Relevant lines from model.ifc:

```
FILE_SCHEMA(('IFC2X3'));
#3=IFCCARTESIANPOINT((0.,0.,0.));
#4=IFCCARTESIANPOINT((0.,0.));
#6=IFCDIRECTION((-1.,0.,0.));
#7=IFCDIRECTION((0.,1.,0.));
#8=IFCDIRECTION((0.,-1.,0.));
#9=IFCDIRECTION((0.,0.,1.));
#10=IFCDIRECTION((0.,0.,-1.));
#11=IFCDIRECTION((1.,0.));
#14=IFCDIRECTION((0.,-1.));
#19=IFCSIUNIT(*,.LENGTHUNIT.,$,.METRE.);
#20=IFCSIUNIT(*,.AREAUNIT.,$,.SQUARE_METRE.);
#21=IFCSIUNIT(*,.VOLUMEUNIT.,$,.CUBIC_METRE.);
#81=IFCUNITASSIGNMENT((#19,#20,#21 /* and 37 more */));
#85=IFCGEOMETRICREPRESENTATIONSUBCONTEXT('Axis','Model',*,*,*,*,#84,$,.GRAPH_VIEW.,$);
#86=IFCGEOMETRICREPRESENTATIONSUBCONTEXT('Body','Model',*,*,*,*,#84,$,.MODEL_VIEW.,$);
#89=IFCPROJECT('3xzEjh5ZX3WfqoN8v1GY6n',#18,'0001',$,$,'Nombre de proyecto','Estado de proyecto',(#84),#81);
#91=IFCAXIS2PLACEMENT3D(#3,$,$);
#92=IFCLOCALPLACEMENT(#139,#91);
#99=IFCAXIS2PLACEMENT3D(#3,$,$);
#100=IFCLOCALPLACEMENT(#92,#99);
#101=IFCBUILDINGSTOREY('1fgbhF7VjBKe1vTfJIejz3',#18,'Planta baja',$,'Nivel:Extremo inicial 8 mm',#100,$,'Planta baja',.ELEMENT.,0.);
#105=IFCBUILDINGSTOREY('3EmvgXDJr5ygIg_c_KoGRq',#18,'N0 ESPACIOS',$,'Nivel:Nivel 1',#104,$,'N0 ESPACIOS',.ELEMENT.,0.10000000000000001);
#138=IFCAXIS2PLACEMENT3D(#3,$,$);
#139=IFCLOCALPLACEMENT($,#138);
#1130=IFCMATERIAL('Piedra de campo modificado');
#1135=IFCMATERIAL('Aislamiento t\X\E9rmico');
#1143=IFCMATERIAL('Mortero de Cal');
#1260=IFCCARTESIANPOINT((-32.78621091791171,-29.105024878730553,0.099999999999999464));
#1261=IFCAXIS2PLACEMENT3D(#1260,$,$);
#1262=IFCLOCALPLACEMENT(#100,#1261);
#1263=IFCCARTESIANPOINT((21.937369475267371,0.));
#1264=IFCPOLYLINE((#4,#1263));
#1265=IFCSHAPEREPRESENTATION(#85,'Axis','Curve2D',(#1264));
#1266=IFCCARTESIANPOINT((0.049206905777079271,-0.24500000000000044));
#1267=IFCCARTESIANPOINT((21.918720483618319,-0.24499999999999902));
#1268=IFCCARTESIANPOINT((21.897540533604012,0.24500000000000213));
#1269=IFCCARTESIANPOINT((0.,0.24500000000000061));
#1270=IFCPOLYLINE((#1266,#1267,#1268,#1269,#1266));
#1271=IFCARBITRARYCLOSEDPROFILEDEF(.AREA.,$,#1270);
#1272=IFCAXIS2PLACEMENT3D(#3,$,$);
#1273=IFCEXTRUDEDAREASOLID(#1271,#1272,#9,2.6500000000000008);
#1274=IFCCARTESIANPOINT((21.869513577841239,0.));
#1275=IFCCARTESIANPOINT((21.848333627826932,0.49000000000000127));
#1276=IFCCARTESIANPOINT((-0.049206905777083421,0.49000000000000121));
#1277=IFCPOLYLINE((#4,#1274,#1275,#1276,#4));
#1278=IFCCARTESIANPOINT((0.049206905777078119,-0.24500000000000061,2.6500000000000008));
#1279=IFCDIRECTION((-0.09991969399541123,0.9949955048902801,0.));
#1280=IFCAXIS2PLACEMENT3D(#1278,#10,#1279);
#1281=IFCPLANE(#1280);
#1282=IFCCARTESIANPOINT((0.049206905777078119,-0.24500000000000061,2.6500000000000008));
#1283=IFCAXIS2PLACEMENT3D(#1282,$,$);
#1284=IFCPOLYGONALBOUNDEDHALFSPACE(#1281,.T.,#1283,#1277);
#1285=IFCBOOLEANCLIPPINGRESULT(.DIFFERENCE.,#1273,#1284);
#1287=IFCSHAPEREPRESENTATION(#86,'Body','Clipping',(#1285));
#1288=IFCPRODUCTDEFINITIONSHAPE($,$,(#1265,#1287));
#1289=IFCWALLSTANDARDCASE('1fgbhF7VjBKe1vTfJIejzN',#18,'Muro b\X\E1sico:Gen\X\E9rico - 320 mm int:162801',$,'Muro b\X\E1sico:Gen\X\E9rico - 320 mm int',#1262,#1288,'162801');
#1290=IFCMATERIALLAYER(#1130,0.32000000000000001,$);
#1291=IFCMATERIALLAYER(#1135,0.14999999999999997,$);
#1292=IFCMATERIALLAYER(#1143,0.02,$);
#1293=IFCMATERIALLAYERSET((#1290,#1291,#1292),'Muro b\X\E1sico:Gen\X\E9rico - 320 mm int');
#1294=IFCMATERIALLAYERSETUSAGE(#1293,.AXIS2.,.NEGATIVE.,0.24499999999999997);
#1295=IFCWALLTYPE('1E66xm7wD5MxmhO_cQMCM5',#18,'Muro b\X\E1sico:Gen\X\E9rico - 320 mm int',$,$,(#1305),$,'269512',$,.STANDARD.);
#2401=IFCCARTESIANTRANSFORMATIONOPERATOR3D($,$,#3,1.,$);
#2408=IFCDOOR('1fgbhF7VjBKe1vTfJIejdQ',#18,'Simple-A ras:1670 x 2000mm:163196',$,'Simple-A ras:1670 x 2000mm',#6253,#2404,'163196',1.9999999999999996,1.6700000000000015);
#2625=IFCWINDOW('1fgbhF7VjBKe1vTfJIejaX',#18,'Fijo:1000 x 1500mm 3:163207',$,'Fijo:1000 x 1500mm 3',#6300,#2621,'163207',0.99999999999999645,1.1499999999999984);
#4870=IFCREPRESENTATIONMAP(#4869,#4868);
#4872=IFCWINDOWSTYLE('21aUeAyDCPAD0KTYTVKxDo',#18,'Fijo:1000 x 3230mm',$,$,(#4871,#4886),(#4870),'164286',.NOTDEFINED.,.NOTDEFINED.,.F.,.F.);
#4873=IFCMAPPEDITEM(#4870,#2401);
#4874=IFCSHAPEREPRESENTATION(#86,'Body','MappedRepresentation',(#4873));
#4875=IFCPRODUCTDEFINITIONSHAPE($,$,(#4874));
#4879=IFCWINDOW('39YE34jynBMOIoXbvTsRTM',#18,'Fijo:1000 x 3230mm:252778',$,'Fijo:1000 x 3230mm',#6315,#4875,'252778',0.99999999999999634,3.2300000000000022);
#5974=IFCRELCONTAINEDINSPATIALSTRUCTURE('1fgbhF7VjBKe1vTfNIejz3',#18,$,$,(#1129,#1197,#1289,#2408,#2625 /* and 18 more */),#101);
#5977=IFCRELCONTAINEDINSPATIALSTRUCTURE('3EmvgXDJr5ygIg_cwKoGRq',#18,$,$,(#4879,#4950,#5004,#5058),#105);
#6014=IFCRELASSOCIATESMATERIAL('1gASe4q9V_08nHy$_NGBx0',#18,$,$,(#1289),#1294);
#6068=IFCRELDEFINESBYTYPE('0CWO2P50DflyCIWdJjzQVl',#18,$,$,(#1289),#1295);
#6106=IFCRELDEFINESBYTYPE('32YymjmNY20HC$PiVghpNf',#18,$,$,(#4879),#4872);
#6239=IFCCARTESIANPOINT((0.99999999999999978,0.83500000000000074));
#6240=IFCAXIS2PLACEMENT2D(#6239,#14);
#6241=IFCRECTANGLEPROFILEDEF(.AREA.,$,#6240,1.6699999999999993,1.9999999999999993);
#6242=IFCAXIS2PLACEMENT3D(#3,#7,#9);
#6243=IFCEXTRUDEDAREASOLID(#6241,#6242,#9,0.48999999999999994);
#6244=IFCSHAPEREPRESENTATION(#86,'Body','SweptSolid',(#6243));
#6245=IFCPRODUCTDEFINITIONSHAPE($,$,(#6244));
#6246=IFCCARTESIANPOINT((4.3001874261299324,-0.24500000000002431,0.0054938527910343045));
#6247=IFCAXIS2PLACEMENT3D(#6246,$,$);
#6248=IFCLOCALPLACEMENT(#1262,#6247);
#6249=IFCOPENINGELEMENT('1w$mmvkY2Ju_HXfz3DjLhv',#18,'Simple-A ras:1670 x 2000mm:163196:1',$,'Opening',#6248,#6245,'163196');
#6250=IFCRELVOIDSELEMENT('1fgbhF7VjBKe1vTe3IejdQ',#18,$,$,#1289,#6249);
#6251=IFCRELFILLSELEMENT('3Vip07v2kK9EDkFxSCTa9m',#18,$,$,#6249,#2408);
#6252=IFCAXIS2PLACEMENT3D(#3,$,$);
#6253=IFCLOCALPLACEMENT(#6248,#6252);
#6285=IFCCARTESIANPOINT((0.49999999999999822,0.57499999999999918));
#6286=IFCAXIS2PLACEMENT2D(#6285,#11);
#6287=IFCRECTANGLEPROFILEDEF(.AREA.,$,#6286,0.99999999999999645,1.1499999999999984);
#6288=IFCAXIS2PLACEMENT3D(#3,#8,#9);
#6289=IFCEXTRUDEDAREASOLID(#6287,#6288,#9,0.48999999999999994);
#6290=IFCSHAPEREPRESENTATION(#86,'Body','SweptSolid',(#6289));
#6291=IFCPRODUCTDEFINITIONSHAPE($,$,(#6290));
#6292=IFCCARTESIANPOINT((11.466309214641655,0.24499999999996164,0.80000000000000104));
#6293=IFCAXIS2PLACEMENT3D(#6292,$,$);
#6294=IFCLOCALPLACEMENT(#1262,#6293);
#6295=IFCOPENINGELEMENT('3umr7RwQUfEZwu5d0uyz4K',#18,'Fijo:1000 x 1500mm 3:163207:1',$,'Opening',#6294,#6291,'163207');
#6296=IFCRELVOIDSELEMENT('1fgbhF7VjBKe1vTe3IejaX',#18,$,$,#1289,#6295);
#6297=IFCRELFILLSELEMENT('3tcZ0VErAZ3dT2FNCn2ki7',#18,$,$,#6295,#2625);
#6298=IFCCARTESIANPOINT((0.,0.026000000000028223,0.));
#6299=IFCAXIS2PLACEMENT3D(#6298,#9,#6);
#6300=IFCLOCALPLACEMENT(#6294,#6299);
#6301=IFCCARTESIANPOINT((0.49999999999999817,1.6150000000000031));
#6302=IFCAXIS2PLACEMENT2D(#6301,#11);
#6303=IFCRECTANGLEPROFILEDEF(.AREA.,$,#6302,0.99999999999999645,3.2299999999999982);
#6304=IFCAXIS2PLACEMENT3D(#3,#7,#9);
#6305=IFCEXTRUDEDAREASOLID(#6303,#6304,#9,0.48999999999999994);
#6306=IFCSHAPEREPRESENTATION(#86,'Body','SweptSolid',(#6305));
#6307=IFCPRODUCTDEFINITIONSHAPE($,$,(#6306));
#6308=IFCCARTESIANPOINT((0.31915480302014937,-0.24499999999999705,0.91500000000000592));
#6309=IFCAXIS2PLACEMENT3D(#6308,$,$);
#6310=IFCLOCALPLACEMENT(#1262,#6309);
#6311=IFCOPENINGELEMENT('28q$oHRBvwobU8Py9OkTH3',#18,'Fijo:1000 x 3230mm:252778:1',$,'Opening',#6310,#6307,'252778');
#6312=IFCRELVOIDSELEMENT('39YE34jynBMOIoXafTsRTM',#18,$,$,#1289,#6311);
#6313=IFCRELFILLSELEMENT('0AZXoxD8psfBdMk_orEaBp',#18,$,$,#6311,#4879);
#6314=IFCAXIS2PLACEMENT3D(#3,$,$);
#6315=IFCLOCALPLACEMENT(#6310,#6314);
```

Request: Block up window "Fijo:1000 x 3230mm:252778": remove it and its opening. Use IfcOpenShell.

```python
import ifcopenshell
import ifcopenshell.api.feature
import ifcopenshell.api.root
import ifcopenshell.geom
import ifcopenshell.util.shape

model = ifcopenshell.open("model.ifc")
settings = ifcopenshell.geom.settings()


def volume(element):
    """Net volume in cubic metres, openings subtracted."""
    shape = ifcopenshell.geom.create_shape(settings, element)
    return ifcopenshell.util.shape.get_volume(shape.geometry)


window = model.by_guid("39YE34jynBMOIoXbvTsRTM")
opening = window.FillsVoids[0].RelatingOpeningElement
wall = opening.VoidsElements[0].RelatingBuildingElement
before = volume(wall)

ifcopenshell.api.root.remove_product(model, product=window)
ifcopenshell.api.feature.remove_feature(model, feature=opening)

after = volume(wall)

print(f"wall volume {before:.3f} -> {after:.3f} m3")

model.write("model_rev.ifc")
```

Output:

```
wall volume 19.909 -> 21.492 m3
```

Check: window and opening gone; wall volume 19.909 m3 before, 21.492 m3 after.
